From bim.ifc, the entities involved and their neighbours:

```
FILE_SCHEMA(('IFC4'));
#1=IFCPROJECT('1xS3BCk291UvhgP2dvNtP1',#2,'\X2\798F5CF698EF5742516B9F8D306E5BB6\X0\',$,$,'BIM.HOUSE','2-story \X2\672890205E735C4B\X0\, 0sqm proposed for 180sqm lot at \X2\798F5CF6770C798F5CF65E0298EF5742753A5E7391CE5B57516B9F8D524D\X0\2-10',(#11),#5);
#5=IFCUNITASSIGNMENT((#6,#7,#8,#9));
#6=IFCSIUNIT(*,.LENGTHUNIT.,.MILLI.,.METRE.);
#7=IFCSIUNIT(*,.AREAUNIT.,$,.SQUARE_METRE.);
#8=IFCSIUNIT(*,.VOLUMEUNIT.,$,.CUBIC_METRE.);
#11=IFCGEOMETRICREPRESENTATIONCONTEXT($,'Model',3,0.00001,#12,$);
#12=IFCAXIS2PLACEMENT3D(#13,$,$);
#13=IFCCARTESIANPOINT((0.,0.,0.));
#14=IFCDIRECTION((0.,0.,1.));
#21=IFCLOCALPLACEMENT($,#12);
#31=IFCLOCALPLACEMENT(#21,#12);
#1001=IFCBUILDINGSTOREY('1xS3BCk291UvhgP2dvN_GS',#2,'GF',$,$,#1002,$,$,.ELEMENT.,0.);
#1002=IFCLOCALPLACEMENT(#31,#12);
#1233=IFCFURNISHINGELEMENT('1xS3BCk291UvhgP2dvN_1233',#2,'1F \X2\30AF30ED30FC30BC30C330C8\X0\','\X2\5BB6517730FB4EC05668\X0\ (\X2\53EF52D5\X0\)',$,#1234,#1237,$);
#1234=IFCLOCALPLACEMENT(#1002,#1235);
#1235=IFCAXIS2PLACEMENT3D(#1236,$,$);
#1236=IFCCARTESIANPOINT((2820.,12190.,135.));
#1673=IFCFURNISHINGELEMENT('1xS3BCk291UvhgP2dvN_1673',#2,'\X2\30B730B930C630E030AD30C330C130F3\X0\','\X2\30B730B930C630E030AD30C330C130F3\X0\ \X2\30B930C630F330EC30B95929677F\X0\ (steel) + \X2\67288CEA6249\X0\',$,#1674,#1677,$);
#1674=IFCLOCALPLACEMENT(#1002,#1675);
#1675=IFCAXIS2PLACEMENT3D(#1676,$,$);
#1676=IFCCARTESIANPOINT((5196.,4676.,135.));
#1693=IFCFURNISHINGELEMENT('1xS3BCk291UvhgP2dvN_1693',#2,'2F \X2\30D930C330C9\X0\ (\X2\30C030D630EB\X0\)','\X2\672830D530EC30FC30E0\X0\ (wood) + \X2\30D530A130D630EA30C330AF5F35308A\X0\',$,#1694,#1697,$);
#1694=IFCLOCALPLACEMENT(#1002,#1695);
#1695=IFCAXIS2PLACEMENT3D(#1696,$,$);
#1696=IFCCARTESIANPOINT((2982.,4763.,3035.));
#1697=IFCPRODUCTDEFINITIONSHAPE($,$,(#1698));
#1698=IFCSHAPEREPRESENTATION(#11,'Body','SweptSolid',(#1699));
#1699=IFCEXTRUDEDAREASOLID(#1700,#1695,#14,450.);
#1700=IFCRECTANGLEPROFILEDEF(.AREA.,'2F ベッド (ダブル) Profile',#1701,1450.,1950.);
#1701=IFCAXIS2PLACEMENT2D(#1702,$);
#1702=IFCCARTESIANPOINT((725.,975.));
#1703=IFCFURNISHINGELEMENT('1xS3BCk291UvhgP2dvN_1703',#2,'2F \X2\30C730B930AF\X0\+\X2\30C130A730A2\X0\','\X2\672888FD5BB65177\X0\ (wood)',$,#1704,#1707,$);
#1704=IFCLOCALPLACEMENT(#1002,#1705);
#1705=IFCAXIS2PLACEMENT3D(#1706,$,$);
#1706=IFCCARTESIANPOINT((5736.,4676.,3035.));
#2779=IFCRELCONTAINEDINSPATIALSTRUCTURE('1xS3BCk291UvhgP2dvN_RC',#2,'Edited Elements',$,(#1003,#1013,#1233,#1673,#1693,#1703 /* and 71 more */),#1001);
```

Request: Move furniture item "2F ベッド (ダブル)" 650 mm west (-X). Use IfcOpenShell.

```python
import ifcopenshell
import ifcopenshell.api.geometry
import ifcopenshell.util.placement

model = ifcopenshell.open("bim.ifc")

item = model.by_guid("1xS3BCk291UvhgP2dvN_1693")
matrix = ifcopenshell.util.placement.get_local_placement(item.ObjectPlacement)
matrix[0, 3] -= 650.0
ifcopenshell.api.geometry.edit_object_placement(model, product=item, matrix=matrix, is_si=False)

print(ifcopenshell.util.placement.get_local_placement(item.ObjectPlacement).round(3) + 0.0)

model.write("bim_v2.ifc")
```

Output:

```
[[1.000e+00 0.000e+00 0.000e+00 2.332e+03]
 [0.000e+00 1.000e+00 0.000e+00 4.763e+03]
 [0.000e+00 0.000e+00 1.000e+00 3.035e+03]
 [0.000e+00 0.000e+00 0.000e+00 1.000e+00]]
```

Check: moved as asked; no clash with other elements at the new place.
